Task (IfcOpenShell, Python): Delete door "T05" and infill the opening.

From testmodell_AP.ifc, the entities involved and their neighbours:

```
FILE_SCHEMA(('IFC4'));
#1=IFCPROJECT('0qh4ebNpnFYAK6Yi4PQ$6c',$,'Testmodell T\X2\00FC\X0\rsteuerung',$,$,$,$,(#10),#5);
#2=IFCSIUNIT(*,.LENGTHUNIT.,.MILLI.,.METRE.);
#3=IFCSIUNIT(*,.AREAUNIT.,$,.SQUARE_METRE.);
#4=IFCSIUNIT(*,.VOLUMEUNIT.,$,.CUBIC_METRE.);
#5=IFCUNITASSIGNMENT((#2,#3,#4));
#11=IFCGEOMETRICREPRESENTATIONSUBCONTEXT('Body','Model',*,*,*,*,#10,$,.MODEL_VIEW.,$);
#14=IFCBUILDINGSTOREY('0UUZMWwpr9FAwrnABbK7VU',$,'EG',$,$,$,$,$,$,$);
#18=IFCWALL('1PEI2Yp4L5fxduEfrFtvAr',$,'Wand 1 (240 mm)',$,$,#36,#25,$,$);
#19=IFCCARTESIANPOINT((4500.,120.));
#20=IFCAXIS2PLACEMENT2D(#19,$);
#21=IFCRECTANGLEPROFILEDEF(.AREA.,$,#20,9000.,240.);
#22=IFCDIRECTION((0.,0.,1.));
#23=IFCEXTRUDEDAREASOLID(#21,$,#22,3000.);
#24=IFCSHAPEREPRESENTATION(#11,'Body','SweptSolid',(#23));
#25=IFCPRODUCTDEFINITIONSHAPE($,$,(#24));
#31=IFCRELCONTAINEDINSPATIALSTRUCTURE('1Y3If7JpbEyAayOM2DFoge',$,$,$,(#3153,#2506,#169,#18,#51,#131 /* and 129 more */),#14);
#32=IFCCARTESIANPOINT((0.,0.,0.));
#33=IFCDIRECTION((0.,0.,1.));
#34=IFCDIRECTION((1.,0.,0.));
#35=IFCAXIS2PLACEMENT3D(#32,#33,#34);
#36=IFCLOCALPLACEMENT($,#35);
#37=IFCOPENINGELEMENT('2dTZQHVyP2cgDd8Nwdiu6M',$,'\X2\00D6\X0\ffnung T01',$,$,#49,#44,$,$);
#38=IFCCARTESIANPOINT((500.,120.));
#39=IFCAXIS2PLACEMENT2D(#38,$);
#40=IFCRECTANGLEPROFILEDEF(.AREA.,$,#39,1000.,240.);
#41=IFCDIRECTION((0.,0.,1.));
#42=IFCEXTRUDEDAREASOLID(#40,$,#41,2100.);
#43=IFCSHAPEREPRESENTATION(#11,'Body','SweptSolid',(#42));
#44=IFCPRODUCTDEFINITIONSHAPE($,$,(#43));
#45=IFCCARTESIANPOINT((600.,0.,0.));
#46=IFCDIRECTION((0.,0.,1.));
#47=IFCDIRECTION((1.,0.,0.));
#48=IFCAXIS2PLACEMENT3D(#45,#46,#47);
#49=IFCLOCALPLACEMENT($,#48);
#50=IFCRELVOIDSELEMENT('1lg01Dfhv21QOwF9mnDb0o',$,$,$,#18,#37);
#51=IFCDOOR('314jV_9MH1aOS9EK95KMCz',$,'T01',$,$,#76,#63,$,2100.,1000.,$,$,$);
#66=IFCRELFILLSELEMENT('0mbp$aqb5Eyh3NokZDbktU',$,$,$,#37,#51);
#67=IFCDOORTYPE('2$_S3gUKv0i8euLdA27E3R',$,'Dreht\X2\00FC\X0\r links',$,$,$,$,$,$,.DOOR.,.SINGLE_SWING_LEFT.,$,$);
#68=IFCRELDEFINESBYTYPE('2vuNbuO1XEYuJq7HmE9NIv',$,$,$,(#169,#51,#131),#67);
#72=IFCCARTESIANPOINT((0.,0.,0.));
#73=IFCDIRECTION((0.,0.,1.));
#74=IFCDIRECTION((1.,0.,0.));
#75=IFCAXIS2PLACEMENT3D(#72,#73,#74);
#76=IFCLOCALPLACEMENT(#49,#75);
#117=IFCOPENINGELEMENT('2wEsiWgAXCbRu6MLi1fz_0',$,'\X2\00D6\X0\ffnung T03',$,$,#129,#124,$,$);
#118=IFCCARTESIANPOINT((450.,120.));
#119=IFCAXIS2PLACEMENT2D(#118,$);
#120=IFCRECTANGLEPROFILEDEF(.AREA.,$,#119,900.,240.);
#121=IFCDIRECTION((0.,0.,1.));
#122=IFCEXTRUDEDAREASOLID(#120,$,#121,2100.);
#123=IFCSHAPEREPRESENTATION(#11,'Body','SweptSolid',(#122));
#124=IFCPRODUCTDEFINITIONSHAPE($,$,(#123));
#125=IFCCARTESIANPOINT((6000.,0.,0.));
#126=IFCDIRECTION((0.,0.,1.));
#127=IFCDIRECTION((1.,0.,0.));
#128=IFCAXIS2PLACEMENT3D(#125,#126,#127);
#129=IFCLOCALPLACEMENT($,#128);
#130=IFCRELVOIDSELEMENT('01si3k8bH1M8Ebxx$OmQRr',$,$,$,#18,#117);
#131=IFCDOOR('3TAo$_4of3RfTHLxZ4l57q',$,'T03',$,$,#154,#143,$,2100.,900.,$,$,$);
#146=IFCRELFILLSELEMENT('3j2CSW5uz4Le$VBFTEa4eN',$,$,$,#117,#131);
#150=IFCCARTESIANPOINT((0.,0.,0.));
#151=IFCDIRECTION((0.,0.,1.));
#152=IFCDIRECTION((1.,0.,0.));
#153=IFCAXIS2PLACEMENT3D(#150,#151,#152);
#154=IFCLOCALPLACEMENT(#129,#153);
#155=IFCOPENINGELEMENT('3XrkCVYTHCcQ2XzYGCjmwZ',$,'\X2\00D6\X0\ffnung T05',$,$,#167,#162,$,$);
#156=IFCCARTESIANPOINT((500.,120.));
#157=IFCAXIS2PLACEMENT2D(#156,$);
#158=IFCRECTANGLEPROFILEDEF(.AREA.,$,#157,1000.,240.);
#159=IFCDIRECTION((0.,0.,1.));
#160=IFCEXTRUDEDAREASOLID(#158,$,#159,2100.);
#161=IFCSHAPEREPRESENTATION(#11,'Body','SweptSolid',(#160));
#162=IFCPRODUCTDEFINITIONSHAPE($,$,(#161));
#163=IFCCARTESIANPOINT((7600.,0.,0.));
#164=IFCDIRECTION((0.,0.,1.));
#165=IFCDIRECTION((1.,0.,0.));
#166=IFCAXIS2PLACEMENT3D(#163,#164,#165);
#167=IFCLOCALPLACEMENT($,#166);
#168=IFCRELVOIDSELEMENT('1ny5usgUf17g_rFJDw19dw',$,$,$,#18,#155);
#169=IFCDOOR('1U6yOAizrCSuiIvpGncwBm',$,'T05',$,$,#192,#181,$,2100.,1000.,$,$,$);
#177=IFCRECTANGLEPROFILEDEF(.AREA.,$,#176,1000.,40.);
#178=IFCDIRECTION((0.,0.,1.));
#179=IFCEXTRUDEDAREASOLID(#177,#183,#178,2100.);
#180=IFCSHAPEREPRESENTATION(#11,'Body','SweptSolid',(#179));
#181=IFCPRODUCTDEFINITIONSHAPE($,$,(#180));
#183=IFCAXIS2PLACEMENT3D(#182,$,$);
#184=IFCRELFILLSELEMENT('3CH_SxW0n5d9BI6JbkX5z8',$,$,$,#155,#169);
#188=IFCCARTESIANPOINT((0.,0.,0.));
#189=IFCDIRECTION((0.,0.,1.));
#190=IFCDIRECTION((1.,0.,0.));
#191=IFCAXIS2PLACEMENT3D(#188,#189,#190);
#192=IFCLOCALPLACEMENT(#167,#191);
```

```python
import ifcopenshell
import ifcopenshell.api.feature
import ifcopenshell.api.root
import ifcopenshell.geom
import ifcopenshell.util.shape

model = ifcopenshell.open("testmodell_AP.ifc")
settings = ifcopenshell.geom.settings()


def volume(element):
    """Net volume in cubic metres, openings subtracted."""
    shape = ifcopenshell.geom.create_shape(settings, element)
    return ifcopenshell.util.shape.get_volume(shape.geometry)


door = model.by_guid("1U6yOAizrCSuiIvpGncwBm")
opening = door.FillsVoids[0].RelatingOpeningElement
wall = opening.VoidsElements[0].RelatingBuildingElement
before = volume(wall)

ifcopenshell.api.root.remove_product(model, product=door)
ifcopenshell.api.feature.remove_feature(model, feature=opening)

after = volume(wall)

print(f"wall volume {before:.3f} -> {after:.3f} m3")

model.write("testmodell_AP_v2.ifc")
```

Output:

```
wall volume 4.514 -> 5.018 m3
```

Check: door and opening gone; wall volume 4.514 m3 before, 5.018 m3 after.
